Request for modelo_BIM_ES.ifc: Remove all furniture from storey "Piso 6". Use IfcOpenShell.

First a look at what the model holds.

```python
import ifcopenshell
import ifcopenshell.util.element

model = ifcopenshell.open("modelo_BIM_ES.ifc")
print(model.schema)
storey = next(s for s in model.by_type("IfcBuildingStorey") if s.Name == "Piso 6")
furniture = [e for e in ifcopenshell.util.element.get_decomposition(storey) if e.is_a("IfcFurnishingElement")]
seen = {}
for e in furniture:
    element_type = ifcopenshell.util.element.get_type(e)
    name = element_type.Name if element_type not in (None, e) else None
    seen[name] = seen.get(name, 0) + 1
for name, count in sorted(seen.items(), key=str):
    print(count, "x", name)
```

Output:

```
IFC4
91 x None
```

```python
import ifcopenshell
import ifcopenshell.api.root
import ifcopenshell.util.element

model = ifcopenshell.open("modelo_BIM_ES.ifc")

storey = next(s for s in model.by_type("IfcBuildingStorey") if s.Name == "Piso 6")
furniture = [e for e in ifcopenshell.util.element.get_decomposition(storey) if e.is_a("IfcFurnishingElement")]

for e in furniture:
    ifcopenshell.api.root.remove_product(model, product=e)
print(len(furniture), "removed")

model.write("modelo_BIM_ES-out.ifc")
```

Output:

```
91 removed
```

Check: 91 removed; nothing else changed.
